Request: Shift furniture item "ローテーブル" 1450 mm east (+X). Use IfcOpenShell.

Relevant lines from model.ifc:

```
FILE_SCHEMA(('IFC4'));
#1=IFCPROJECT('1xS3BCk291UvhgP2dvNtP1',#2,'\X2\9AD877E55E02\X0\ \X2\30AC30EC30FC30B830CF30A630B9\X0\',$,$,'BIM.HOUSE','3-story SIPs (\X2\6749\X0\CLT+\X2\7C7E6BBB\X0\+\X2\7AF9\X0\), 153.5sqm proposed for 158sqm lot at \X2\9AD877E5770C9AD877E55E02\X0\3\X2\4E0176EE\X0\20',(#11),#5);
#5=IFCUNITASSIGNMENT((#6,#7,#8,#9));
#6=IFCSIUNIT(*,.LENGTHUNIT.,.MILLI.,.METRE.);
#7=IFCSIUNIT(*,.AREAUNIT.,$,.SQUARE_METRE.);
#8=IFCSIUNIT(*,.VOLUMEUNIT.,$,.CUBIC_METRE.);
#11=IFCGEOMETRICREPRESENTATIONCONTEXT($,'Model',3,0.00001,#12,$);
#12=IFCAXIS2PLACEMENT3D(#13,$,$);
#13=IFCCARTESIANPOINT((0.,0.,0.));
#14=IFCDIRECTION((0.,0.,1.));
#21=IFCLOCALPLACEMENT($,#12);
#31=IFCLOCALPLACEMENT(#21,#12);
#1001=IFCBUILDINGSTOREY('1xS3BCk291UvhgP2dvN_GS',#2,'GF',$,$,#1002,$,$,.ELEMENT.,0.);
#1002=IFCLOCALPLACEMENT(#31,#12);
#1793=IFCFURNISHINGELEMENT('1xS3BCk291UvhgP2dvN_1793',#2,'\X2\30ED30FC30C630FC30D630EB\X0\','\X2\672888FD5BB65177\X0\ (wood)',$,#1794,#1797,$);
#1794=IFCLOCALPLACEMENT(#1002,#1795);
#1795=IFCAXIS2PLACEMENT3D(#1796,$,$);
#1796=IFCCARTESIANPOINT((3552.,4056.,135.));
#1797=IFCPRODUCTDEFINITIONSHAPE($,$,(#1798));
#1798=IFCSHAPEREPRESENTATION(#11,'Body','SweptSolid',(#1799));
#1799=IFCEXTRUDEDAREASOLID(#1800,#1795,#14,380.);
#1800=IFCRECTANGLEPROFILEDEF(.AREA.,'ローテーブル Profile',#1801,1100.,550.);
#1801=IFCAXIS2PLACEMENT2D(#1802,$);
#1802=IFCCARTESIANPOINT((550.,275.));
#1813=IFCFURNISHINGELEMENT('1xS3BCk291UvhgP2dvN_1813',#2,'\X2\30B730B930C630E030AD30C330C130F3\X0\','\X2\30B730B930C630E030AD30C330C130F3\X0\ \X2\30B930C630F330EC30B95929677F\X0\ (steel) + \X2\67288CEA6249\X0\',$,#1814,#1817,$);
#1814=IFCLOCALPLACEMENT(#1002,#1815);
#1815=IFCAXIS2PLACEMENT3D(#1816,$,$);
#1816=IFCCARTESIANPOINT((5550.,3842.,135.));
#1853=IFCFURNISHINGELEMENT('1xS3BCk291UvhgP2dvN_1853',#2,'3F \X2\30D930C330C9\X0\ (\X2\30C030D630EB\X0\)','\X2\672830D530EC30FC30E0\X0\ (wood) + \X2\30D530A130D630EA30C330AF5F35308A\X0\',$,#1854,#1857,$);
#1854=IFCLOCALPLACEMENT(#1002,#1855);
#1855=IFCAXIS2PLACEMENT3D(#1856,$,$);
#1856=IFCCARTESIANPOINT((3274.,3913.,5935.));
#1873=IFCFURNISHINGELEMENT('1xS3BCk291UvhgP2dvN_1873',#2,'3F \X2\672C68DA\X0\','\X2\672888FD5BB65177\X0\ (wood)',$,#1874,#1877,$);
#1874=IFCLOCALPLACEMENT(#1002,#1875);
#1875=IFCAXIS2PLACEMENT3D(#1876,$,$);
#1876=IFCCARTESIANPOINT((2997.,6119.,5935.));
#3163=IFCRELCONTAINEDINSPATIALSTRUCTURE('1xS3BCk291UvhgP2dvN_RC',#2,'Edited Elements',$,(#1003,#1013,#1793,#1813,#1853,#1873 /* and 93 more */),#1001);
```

```python
import ifcopenshell
import ifcopenshell.api.geometry
import ifcopenshell.util.placement
import ifcopenshell.util.unit

model = ifcopenshell.open("model.ifc")
unit_scale = ifcopenshell.util.unit.calculate_unit_scale(model)

item = model.by_id(1793)
matrix = ifcopenshell.util.placement.get_local_placement(item.ObjectPlacement)
matrix[0, 3] += 1.45 / unit_scale
ifcopenshell.api.geometry.edit_object_placement(model, product=item, matrix=matrix, is_si=False)

print(ifcopenshell.util.placement.get_local_placement(item.ObjectPlacement).round(3) + 0.0)

model.write("model_updated.ifc")
```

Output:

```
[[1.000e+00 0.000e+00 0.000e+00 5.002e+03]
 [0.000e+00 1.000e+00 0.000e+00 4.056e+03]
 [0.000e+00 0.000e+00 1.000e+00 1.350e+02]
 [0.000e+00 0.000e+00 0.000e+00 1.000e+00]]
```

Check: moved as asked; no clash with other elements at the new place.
